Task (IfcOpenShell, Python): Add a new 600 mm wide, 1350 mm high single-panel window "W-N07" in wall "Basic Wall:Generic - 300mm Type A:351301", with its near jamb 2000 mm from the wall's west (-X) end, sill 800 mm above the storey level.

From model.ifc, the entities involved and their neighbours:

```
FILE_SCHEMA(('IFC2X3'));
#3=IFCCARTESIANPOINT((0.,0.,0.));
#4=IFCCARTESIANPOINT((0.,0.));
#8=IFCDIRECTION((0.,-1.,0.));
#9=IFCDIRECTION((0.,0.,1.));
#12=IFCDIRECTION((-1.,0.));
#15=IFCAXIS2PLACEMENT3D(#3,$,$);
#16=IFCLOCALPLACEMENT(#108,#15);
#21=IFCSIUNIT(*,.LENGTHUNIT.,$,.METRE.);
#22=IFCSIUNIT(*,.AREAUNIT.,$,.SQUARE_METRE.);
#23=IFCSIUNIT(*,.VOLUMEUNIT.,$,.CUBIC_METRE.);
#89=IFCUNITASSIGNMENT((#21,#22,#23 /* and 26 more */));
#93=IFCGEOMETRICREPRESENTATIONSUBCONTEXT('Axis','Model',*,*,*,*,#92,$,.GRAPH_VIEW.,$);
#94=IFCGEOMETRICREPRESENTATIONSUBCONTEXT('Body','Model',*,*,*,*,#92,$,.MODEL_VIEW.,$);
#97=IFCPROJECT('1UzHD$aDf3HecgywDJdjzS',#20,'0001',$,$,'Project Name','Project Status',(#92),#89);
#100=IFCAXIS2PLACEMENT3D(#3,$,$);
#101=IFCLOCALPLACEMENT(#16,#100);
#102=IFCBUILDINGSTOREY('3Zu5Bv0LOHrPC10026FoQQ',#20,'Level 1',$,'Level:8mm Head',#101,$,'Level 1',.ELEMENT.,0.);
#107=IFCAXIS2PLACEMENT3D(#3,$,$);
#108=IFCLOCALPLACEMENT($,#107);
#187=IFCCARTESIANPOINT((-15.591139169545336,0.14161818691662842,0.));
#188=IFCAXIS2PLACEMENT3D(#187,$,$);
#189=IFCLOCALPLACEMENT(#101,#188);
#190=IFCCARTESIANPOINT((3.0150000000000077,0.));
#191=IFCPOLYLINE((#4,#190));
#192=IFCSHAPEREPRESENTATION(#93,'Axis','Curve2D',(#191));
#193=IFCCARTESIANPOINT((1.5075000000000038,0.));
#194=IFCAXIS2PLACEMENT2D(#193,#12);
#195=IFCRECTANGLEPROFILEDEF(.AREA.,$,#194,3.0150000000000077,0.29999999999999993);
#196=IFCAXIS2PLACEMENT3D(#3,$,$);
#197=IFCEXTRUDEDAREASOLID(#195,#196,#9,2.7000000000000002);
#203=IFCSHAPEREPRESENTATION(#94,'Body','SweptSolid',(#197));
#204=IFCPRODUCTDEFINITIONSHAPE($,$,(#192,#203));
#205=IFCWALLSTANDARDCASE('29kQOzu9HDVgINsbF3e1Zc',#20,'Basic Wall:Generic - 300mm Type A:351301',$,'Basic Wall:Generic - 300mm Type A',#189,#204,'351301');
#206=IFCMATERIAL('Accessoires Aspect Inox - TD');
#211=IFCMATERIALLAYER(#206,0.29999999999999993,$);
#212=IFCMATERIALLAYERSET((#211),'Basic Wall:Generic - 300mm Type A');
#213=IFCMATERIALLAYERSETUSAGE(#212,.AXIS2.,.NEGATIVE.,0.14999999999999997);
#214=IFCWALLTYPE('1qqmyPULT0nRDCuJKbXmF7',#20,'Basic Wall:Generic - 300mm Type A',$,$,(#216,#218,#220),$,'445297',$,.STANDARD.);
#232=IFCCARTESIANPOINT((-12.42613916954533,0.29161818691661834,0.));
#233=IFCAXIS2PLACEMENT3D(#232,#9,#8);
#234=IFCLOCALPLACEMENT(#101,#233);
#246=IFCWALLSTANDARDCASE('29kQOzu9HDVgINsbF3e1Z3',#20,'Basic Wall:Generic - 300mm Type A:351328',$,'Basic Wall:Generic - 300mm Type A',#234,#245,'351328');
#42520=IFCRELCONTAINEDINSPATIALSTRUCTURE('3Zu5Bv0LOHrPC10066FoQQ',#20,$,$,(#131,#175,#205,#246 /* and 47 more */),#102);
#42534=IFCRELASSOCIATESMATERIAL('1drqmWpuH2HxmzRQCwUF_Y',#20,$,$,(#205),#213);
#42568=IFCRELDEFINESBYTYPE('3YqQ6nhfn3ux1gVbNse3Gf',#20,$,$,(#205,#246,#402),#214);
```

```python
import numpy as np
import ifcopenshell
import ifcopenshell.api.feature
import ifcopenshell.api.geometry
import ifcopenshell.api.root
import ifcopenshell.api.spatial
import ifcopenshell.api.type
import ifcopenshell.geom
import ifcopenshell.util.element
import ifcopenshell.util.placement
import ifcopenshell.util.representation
import ifcopenshell.util.shape
import ifcopenshell.util.unit

model = ifcopenshell.open("model.ifc")
unit_scale = ifcopenshell.util.unit.calculate_unit_scale(model)
settings = ifcopenshell.geom.settings()


def volume(element):
    """Net volume in cubic metres, openings subtracted."""
    shape = ifcopenshell.geom.create_shape(settings, element)
    return ifcopenshell.util.shape.get_volume(shape.geometry)


wall = model.by_guid("29kQOzu9HDVgINsbF3e1Zc")
storey = ifcopenshell.util.element.get_container(wall, ifc_class="IfcBuildingStorey")
context = ifcopenshell.util.representation.get_context(model, "Model", "Body", "MODEL_VIEW")
before = volume(wall)

width, height, from_end, sill = 0.6, 1.35, 2, 0.8  # metres

# The wall runs along its own X axis, and the end named is its -X end.
wall_shape = ifcopenshell.geom.create_shape(settings, wall)
x, y, z = ifcopenshell.util.shape.get_vertices(wall_shape.geometry).T
start = x.min() + from_end
face, thickness = float(y.min()), float(y.max() - y.min())
wall_matrix = ifcopenshell.util.placement.get_local_placement(wall.ObjectPlacement)
level = ifcopenshell.util.placement.get_local_placement(storey.ObjectPlacement)[2, 3]


def in_wall(x, y):
    """Placement at x, y metres in the wall's axes, at sill height."""
    matrix = wall_matrix.copy()
    matrix[:, 3] = wall_matrix @ np.array([x / unit_scale, y / unit_scale, 0.0, 1.0])
    matrix[2, 3] = level + sill / unit_scale
    return matrix


# Opening: a box that overshoots both wall faces by 50 mm.
opening = ifcopenshell.api.root.create_entity(model, ifc_class="IfcOpeningElement")
box = ifcopenshell.api.geometry.add_wall_representation(
    model, context=context, length=width, height=height, thickness=thickness + 0.1
)
ifcopenshell.api.geometry.assign_representation(model, product=opening, representation=box)
ifcopenshell.api.geometry.edit_object_placement(model, product=opening, matrix=in_wall(start, face - 0.05), is_si=False)
ifcopenshell.api.feature.add_feature(model, feature=opening, element=wall)

window = ifcopenshell.api.root.create_entity(model, ifc_class="IfcWindow", name="W-N07")
window.OverallWidth, window.OverallHeight = width / unit_scale, height / unit_scale
body = ifcopenshell.api.geometry.add_window_representation(
    model,
    context=context,
    overall_width=window.OverallWidth,
    overall_height=window.OverallHeight,
    partition_type="SINGLE_PANEL",
)
ifcopenshell.api.geometry.assign_representation(model, product=window, representation=body)
ifcopenshell.api.spatial.assign_container(model, products=[window], relating_structure=storey)
fills = ifcopenshell.api.feature.add_filling(model, opening=opening, element=window)
fills.OwnerHistory = window.OwnerHistory  # required in IFC2X3

# IFC2X3 keeps the operation on the window style.
style = ifcopenshell.api.root.create_entity(model, ifc_class="IfcWindowStyle", name="W-N07")
style.OperationType, style.ConstructionType = "SINGLE_PANEL", "NOTDEFINED"
style.ParameterTakesPrecedence = style.Sizeable = False
ifcopenshell.api.type.assign_type(model, related_objects=[window], relating_type=style)

# Centre the window in the wall's thickness.
ifcopenshell.api.geometry.edit_object_placement(model, product=window, matrix=in_wall(start, face), is_si=False)
window_shape = ifcopenshell.geom.create_shape(settings, window)
depth = ifcopenshell.util.shape.get_vertices(window_shape.geometry)[:, 1]
offset = face + thickness / 2 - (depth.min() + depth.max()) / 2
ifcopenshell.api.geometry.edit_object_placement(model, product=window, matrix=in_wall(start, offset), is_si=False)

after = volume(wall)

print(f"wall volume {before:.3f} -> {after:.3f} m3")

model.write("model_edited.ifc")
```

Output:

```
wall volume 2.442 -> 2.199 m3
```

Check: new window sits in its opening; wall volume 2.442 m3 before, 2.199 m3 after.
